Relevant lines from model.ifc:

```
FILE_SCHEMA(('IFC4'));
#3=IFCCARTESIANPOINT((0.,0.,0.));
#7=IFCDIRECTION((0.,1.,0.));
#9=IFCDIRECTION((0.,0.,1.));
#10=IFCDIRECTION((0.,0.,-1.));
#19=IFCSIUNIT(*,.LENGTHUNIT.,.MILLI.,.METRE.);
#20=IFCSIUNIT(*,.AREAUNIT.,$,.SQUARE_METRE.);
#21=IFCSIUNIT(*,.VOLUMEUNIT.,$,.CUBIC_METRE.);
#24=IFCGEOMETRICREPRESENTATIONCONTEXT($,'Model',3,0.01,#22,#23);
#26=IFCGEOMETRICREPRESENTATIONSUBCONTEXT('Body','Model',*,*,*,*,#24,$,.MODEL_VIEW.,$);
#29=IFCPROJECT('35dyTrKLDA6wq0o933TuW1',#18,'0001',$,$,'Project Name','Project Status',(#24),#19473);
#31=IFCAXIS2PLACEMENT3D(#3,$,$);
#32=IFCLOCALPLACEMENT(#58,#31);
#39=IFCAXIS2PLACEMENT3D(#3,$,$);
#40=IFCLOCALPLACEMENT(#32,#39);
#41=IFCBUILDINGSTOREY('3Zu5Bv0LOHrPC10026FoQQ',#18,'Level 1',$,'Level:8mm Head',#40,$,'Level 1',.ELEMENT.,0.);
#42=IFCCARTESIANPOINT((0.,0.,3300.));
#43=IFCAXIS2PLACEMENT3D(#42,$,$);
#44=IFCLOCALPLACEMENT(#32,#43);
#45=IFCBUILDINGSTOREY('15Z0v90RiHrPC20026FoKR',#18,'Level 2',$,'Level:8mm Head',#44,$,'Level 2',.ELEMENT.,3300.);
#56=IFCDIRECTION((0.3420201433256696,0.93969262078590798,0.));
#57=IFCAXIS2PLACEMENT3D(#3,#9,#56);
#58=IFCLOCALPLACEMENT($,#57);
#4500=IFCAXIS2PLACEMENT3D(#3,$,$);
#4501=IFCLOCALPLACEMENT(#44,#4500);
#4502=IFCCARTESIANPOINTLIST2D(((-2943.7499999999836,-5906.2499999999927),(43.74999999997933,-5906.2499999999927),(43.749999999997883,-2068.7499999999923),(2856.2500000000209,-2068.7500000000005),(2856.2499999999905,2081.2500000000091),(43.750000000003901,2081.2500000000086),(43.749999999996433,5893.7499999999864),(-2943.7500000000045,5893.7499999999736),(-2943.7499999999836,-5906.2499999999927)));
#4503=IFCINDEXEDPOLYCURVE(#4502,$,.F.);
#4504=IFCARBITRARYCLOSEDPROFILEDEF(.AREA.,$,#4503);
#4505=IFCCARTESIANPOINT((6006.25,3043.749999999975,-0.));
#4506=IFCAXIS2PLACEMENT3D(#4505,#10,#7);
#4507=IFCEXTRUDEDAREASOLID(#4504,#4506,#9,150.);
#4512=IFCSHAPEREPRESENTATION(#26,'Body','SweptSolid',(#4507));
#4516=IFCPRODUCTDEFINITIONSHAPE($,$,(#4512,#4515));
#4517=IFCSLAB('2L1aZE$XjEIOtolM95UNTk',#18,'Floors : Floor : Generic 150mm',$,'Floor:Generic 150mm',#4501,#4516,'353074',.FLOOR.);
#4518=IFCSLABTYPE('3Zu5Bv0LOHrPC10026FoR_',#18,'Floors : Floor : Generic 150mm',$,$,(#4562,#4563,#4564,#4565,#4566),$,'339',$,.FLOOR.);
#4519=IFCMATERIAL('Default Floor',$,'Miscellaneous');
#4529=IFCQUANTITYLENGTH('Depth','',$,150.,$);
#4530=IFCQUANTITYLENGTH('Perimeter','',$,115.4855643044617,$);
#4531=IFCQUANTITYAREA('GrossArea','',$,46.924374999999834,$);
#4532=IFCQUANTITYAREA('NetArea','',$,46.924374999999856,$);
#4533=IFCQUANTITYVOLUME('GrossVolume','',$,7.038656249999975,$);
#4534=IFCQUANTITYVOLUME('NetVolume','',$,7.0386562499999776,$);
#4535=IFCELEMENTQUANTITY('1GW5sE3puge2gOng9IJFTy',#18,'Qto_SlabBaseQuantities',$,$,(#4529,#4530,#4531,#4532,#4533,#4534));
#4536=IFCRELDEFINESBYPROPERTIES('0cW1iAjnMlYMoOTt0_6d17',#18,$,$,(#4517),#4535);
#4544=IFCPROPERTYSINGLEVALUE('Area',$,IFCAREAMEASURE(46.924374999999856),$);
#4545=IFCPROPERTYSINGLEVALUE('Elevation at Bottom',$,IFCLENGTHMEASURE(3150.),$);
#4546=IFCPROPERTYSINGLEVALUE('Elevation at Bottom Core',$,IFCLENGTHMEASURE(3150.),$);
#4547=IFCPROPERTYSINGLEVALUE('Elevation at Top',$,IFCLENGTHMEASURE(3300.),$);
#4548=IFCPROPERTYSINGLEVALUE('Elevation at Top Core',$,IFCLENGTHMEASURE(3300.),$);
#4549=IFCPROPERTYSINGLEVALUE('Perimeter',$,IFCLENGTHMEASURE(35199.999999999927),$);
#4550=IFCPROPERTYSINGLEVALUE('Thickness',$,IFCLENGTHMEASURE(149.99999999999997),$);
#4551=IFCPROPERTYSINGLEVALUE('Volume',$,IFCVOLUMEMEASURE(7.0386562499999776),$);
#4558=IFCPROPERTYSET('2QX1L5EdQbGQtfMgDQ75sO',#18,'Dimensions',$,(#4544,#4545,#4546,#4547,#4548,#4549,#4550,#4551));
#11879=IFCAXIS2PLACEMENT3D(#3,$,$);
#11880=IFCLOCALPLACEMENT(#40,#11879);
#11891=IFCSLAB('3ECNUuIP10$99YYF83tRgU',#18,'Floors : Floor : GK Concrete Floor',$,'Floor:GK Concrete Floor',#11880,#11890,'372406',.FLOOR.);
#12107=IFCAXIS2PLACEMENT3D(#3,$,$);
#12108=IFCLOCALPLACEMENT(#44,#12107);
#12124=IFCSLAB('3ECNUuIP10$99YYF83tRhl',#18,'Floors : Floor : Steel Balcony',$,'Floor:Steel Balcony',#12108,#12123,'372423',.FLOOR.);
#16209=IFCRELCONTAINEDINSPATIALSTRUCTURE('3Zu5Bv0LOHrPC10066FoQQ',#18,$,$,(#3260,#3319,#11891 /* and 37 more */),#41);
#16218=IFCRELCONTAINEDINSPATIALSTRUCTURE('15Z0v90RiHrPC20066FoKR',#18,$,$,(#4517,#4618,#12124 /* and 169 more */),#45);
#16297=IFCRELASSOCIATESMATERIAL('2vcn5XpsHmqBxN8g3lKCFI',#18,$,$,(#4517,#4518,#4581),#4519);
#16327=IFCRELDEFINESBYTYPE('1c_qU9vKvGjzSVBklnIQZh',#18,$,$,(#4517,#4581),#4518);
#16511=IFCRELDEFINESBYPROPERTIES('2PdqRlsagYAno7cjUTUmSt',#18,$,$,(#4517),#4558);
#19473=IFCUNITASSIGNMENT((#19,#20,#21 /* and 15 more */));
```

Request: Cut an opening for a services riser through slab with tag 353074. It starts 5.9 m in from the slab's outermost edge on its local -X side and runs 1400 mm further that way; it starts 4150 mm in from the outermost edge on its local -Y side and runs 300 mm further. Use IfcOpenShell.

```python
import numpy as np
import ifcopenshell
import ifcopenshell.api.feature
import ifcopenshell.api.geometry
import ifcopenshell.api.pset
import ifcopenshell.api.root
import ifcopenshell.geom
import ifcopenshell.util.element
import ifcopenshell.util.placement
import ifcopenshell.util.representation
import ifcopenshell.util.shape
import ifcopenshell.util.unit

model = ifcopenshell.open("model.ifc")
unit_scale = ifcopenshell.util.unit.calculate_unit_scale(model)
area_scale = ifcopenshell.util.unit.calculate_unit_scale(model, "AREAUNIT")
volume_scale = ifcopenshell.util.unit.calculate_unit_scale(model, "VOLUMEUNIT")
settings = ifcopenshell.geom.settings()


def volume(element):
    """Net volume in cubic metres, openings subtracted."""
    shape = ifcopenshell.geom.create_shape(settings, element)
    return ifcopenshell.util.shape.get_volume(shape.geometry)


slab = model.by_guid("2L1aZE$XjEIOtolM95UNTk")
before = volume(slab)

# Extent in the slab's own axes, in metres. The edges named are its -X and -Y sides.
slab_shape = ifcopenshell.geom.create_shape(settings, slab)
vertices = ifcopenshell.util.shape.get_vertices(slab_shape.geometry)
x_min, y_min, bottom = vertices.min(axis=0)
top = vertices[:, 2].max()

opening = ifcopenshell.api.root.create_entity(model, ifc_class="IfcOpeningElement", name="Services riser opening", predefined_type="OPENING")
context = ifcopenshell.util.representation.get_context(model, "Model", "Body", "MODEL_VIEW")
width, depth = 1.4, 0.3
outline = [(0.0, 0.0), (width, 0.0), (width, depth), (0.0, depth), (0.0, 0.0)]
# Overshoot both faces by 50 mm so the cut is clean.
shape = ifcopenshell.api.geometry.add_slab_representation(
    model, context=context, depth=top - bottom + 0.1, polyline=outline
)
ifcopenshell.api.geometry.assign_representation(model, product=opening, representation=shape)

matrix = ifcopenshell.util.placement.get_local_placement(slab.ObjectPlacement)
matrix[:, 3] = matrix @ np.append(np.array([x_min + 5.9, y_min + 4.15, bottom - 0.05]) / unit_scale, 1.0)
ifcopenshell.api.geometry.edit_object_placement(model, product=opening, matrix=matrix, is_si=False)
ifcopenshell.api.feature.add_feature(model, feature=opening, element=slab)

after = volume(slab)

# Update the slab's stored quantities.
qto = model.by_id(ifcopenshell.util.element.get_pset(slab, "Qto_SlabBaseQuantities", should_inherit=False)["id"])
ifcopenshell.api.pset.edit_qto(model, qto=qto, properties={
    "NetArea": after / (top - bottom) / area_scale,
    "NetVolume": after / volume_scale,
})
pset = model.by_id(ifcopenshell.util.element.get_pset(slab, "Dimensions", should_inherit=False)["id"])
ifcopenshell.api.pset.edit_pset(model, pset=pset, properties={
    "Area": model.create_entity("IfcAreaMeasure", after / (top - bottom) / area_scale),
    "Volume": model.create_entity("IfcVolumeMeasure", after / volume_scale),
})

print(f"slab volume {before:.3f} -> {after:.3f} m3")

model.write("model_updated.ifc")
```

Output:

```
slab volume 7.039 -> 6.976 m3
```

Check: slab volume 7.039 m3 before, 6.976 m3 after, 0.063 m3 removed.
